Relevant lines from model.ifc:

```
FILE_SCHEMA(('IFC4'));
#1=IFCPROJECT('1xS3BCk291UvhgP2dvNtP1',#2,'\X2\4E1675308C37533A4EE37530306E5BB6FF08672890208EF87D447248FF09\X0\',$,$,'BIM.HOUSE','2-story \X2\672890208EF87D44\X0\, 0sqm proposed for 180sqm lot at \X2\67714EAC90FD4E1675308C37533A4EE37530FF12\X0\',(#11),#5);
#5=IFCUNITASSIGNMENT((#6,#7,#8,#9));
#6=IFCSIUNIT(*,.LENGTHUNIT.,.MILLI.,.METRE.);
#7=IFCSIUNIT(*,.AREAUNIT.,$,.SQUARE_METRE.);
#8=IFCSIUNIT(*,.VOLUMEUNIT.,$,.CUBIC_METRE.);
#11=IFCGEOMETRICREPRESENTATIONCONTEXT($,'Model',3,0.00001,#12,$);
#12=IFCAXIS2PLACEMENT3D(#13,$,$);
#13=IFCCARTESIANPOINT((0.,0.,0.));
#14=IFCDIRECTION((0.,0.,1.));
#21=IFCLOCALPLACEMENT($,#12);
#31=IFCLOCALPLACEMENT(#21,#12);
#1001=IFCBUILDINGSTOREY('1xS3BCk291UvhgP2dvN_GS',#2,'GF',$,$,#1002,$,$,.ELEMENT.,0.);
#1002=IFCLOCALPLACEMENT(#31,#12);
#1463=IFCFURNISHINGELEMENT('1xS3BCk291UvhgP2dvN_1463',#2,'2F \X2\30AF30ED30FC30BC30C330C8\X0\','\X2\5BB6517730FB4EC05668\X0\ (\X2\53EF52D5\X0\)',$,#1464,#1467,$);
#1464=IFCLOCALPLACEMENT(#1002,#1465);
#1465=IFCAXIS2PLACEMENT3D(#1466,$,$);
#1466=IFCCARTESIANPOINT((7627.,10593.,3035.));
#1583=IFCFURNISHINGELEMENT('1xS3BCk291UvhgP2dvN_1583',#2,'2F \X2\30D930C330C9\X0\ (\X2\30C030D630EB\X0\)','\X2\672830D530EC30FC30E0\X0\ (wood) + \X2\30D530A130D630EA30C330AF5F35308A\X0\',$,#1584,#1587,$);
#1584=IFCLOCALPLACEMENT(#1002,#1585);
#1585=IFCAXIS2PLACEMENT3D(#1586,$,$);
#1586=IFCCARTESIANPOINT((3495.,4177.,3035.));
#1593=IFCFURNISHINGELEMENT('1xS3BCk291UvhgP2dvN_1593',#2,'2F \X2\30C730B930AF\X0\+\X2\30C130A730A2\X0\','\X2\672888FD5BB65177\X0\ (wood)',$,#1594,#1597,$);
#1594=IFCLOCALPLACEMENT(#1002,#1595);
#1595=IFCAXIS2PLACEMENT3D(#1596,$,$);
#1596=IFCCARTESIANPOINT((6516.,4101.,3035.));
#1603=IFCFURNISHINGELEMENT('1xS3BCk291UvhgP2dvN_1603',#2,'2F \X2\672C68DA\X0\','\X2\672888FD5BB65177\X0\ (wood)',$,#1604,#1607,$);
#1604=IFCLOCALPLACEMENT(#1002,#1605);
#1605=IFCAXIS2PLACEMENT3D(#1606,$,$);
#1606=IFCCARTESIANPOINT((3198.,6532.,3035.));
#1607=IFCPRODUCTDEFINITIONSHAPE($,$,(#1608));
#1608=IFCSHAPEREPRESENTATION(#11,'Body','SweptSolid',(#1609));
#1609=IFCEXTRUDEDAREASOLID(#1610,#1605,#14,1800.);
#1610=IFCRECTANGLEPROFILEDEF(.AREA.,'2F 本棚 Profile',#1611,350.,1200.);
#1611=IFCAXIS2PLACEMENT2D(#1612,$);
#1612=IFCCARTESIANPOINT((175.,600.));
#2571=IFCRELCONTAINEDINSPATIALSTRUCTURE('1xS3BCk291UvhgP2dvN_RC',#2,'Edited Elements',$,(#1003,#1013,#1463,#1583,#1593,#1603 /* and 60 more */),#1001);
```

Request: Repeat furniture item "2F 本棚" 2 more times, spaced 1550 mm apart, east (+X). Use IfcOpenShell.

```python
import numpy as np
import ifcopenshell
import ifcopenshell.api.geometry
import ifcopenshell.api.root
import ifcopenshell.util.element
import ifcopenshell.util.placement

model = ifcopenshell.open("model.ifc")


def reuse_history(source, copy):
    """copy_class also copies each property set's owner history, people and application; keep the originals."""
    for rel in copy.IsDefinedBy:
        if rel.is_a("IfcRelDefinesByProperties") and (history := rel.RelatingPropertyDefinition.OwnerHistory):
            rel.RelatingPropertyDefinition.OwnerHistory = source.OwnerHistory
            ifcopenshell.util.element.remove_deep2(model, history)


source = model.by_guid("1xS3BCk291UvhgP2dvN_1603")
base = ifcopenshell.util.placement.get_local_placement(source.ObjectPlacement)
step = np.array([1.0, 0.0, 0.0]) * 1550.0

for i in range(1, 3):
    copy = ifcopenshell.api.root.copy_class(model, product=source)
    copy.Representation = ifcopenshell.util.element.copy_deep(
        model, source.Representation, exclude=["IfcGeometricRepresentationContext", "IfcRepresentationMap"]
    )
    reuse_history(source, copy)
    matrix = base.copy()
    matrix[:3, 3] += i * step
    print("added at", matrix[:3, 3].round(3) + 0.0)
    ifcopenshell.api.geometry.edit_object_placement(model, product=copy, matrix=matrix, is_si=False)

model.write("model_rev.ifc")
```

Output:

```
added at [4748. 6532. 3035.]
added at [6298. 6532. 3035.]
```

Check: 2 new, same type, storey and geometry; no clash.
